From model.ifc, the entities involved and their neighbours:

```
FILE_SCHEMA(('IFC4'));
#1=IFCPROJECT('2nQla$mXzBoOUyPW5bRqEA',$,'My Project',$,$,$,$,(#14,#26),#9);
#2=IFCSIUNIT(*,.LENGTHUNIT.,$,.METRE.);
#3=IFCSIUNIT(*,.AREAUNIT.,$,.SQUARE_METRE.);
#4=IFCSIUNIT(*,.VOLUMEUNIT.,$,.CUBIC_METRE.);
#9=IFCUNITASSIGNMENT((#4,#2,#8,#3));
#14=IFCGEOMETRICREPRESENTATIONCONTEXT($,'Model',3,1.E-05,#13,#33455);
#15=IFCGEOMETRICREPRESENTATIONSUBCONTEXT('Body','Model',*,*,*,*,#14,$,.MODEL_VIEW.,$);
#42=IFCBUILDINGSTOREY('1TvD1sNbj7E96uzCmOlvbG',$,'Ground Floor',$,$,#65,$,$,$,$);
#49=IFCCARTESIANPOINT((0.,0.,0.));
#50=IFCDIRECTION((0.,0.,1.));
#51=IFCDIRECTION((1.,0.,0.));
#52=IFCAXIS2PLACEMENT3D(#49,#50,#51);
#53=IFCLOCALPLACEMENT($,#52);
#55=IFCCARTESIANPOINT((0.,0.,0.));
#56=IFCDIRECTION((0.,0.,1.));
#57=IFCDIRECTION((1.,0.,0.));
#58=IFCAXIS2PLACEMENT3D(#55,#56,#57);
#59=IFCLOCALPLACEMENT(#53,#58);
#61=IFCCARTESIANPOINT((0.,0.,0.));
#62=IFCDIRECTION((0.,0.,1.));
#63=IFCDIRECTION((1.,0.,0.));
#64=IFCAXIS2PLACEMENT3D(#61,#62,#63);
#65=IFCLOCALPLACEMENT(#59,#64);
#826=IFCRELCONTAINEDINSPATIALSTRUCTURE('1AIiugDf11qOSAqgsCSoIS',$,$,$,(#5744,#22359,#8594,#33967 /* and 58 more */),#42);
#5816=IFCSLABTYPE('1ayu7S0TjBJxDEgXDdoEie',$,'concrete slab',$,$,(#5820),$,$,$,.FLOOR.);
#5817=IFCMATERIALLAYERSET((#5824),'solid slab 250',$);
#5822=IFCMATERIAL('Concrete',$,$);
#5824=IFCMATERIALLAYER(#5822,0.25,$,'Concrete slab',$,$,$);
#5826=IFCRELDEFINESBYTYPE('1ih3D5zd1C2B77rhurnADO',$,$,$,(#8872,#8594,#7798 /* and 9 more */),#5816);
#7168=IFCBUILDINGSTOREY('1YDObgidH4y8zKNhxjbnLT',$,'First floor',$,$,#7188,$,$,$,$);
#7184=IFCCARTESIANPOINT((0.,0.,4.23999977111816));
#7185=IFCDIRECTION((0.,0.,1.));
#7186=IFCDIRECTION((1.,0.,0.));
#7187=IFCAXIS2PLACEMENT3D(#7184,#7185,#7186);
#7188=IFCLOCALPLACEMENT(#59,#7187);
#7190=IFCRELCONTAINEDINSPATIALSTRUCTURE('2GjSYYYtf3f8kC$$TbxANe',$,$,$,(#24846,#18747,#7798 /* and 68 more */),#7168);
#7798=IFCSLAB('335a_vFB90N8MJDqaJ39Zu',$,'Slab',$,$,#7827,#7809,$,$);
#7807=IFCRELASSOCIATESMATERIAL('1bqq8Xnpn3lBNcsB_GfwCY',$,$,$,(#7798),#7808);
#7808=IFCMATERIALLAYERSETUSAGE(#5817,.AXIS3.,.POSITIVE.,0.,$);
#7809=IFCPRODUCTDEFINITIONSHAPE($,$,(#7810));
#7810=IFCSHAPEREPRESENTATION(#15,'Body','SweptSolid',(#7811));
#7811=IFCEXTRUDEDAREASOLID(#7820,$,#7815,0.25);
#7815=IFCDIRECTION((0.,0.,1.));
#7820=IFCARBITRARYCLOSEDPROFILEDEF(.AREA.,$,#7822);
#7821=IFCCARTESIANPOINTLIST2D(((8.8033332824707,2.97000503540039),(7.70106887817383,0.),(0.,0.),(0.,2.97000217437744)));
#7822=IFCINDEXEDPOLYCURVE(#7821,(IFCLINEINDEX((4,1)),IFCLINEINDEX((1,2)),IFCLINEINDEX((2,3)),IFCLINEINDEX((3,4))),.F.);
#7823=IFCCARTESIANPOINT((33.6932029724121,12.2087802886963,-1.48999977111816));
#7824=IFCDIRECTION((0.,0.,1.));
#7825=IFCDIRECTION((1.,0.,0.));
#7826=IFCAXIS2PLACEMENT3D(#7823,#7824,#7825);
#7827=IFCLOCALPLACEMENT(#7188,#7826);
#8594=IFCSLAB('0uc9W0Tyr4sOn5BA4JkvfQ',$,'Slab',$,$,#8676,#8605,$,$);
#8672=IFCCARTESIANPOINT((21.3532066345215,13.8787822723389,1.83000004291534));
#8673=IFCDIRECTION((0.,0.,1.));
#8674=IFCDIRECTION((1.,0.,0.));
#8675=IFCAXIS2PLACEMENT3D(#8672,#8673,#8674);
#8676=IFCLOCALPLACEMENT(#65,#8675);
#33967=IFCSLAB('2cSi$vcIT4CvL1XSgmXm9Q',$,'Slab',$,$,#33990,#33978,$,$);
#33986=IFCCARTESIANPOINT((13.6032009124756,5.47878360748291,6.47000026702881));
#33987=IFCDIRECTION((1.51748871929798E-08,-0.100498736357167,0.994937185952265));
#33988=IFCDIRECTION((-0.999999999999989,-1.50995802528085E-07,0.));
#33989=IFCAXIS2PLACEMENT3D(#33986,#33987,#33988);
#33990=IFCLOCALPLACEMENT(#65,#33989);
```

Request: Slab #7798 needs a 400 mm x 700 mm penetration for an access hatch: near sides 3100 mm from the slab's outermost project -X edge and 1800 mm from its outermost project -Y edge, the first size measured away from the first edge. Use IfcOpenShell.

```python
import numpy as np
import ifcopenshell
import ifcopenshell.api.feature
import ifcopenshell.api.geometry
import ifcopenshell.api.root
import ifcopenshell.geom
import ifcopenshell.util.placement
import ifcopenshell.util.representation
import ifcopenshell.util.shape
import ifcopenshell.util.unit

model = ifcopenshell.open("model.ifc")
unit_scale = ifcopenshell.util.unit.calculate_unit_scale(model)
settings = ifcopenshell.geom.settings()


def volume(element):
    """Net volume in cubic metres, openings subtracted."""
    shape = ifcopenshell.geom.create_shape(settings, element)
    return ifcopenshell.util.shape.get_volume(shape.geometry)


slab = model.by_id(7798)
before = volume(slab)

# Extent in the slab's own axes, in metres. The edges named are its -X and -Y sides.
slab_shape = ifcopenshell.geom.create_shape(settings, slab)
vertices = ifcopenshell.util.shape.get_vertices(slab_shape.geometry)
x_min, y_min, bottom = vertices.min(axis=0)
top = vertices[:, 2].max()

opening = ifcopenshell.api.root.create_entity(model, ifc_class="IfcOpeningElement", name="Access hatch opening", predefined_type="OPENING")
context = ifcopenshell.util.representation.get_context(model, "Model", "Body", "MODEL_VIEW")
width, depth = 0.4, 0.7
outline = [(0.0, 0.0), (width, 0.0), (width, depth), (0.0, depth), (0.0, 0.0)]
# Overshoot both faces by 50 mm so the cut is clean.
shape = ifcopenshell.api.geometry.add_slab_representation(
    model, context=context, depth=top - bottom + 0.1, polyline=outline
)
ifcopenshell.api.geometry.assign_representation(model, product=opening, representation=shape)

matrix = ifcopenshell.util.placement.get_local_placement(slab.ObjectPlacement)
matrix[:, 3] = matrix @ np.append(np.array([x_min + 3.1, y_min + 1.8, bottom - 0.05]) / unit_scale, 1.0)
ifcopenshell.api.geometry.edit_object_placement(model, product=opening, matrix=matrix, is_si=False)
ifcopenshell.api.feature.add_feature(model, feature=opening, element=slab)

after = volume(slab)

print(f"slab volume {before:.3f} -> {after:.3f} m3")

model.write("model_edited.ifc")
```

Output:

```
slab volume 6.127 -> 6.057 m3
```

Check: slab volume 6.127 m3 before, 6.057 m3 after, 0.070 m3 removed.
